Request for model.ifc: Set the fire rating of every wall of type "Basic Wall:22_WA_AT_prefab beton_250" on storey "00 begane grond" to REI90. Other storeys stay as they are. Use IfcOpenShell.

First a look at what the model holds.

```python
import ifcopenshell
import ifcopenshell.util.element

model = ifcopenshell.open("model.ifc")
print(model.schema)
storey = next(s for s in model.by_type("IfcBuildingStorey") if s.Name == "00 begane grond")
walls = [e for e in ifcopenshell.util.element.get_decomposition(storey) if e.is_a("IfcWall")]
seen = {}
for e in walls:
    element_type = ifcopenshell.util.element.get_type(e)
    key = (element_type.Name if element_type != e and element_type else None, ifcopenshell.util.element.get_pset(e, "Pset_WallCommon", "FireRating"))
    seen[key] = seen.get(key, 0) + 1
for (name, value), count in sorted(seen.items(), key=str):
    print(count, "x", name, "|", value)
```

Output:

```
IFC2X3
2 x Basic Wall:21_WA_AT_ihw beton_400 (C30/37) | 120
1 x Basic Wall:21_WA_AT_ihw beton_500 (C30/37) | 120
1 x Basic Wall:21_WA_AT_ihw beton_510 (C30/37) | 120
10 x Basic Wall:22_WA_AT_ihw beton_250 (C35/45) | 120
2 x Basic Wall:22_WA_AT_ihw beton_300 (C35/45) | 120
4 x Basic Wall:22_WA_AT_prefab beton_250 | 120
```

```python
import ifcopenshell
import ifcopenshell.api.pset
import ifcopenshell.util.element

model = ifcopenshell.open("model.ifc")

storey = next(s for s in model.by_type("IfcBuildingStorey") if s.Name == "00 begane grond")
walls = [e for e in ifcopenshell.util.element.get_decomposition(storey) if e.is_a("IfcWall")]

count = 0
for e in walls:
    element_type = ifcopenshell.util.element.get_type(e)
    if element_type in (None, e) or element_type.Name != "Basic Wall:22_WA_AT_prefab beton_250":
        continue
    # add_pset returns the element's existing set when there is one.
    pset = ifcopenshell.api.pset.add_pset(model, product=e, name="Pset_WallCommon")
    ifcopenshell.api.pset.edit_pset(model, pset=pset, properties={"FireRating": "REI90"})
    count += 1

print(count, "walls updated")

model.write("model_updated.ifc")
```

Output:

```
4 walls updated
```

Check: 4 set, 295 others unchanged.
